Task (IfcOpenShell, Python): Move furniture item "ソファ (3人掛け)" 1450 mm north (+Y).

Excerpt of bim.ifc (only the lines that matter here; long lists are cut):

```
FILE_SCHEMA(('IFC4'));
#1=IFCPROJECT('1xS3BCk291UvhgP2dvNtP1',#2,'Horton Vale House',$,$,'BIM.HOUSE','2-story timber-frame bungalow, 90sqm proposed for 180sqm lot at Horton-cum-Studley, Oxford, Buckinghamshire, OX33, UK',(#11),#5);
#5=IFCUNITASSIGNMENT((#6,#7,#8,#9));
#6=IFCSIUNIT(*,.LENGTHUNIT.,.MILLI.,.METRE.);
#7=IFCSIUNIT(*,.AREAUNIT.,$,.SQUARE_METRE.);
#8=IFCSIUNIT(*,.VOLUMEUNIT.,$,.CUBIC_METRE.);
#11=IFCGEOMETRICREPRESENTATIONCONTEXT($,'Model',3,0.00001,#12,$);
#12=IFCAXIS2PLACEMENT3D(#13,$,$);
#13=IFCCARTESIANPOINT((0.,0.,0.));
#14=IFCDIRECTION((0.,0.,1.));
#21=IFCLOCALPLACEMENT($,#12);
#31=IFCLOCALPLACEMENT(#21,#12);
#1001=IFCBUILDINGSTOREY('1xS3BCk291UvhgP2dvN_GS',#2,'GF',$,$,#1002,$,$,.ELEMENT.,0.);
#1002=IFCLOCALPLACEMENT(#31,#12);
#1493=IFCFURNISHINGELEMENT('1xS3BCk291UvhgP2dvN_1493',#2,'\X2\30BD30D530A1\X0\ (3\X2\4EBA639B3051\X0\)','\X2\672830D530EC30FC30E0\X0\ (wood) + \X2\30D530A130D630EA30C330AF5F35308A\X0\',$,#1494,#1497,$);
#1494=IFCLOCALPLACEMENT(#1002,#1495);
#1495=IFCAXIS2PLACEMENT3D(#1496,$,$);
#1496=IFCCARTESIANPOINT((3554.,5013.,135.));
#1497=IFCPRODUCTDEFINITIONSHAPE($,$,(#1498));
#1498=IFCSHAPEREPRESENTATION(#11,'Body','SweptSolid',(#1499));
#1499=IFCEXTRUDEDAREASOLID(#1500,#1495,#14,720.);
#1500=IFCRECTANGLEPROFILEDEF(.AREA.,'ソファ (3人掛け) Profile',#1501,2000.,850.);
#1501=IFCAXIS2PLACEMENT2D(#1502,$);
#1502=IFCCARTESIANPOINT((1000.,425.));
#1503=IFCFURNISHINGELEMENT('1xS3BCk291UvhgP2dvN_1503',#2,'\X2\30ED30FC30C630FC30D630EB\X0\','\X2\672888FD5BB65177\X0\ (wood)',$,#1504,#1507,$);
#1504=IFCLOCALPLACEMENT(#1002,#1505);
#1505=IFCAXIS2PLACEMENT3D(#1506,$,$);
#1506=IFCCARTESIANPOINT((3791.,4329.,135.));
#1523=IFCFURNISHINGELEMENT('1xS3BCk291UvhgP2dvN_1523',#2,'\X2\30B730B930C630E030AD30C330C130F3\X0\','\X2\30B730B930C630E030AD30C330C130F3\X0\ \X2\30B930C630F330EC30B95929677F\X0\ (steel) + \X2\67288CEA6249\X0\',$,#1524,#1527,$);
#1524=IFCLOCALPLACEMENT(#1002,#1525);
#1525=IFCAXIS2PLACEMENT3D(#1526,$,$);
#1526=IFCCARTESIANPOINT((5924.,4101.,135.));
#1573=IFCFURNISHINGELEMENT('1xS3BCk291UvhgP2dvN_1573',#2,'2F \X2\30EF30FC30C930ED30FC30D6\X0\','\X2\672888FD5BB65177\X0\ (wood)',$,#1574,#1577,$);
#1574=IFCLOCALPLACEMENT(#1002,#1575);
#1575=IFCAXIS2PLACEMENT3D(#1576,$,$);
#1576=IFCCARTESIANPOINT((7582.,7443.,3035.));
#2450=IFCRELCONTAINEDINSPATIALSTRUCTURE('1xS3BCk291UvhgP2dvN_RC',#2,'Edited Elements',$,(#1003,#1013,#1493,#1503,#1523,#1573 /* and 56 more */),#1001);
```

```python
import ifcopenshell
import ifcopenshell.api.geometry
import ifcopenshell.util.placement
import ifcopenshell.util.unit

model = ifcopenshell.open("bim.ifc")
unit_scale = ifcopenshell.util.unit.calculate_unit_scale(model)

item = model.by_guid("1xS3BCk291UvhgP2dvN_1493")
matrix = ifcopenshell.util.placement.get_local_placement(item.ObjectPlacement)
matrix[1, 3] += 1.45 / unit_scale
ifcopenshell.api.geometry.edit_object_placement(model, product=item, matrix=matrix, is_si=False)

print(ifcopenshell.util.placement.get_local_placement(item.ObjectPlacement).round(3) + 0.0)

model.write("bim_updated.ifc")
```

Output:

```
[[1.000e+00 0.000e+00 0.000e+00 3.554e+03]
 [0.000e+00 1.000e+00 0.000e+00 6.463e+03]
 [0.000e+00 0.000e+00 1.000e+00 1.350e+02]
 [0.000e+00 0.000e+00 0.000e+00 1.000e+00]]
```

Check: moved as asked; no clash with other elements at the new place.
